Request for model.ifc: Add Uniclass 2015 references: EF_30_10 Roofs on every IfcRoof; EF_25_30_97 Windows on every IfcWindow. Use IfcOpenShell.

First a look at what the model holds.

```python
import ifcopenshell

model = ifcopenshell.open("model.ifc")
print(model.schema)
print("classifications:", [c.Name for c in model.by_type("IfcClassification")])
for ifc_class in ("IfcDoor", "IfcRoof", "IfcStair", "IfcWall", "IfcWindow"):
    print(ifc_class, len(model.by_type(ifc_class)))
```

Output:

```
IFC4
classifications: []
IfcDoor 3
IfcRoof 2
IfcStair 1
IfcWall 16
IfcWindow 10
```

```python
import ifcopenshell
import ifcopenshell.api.classification

model = ifcopenshell.open("model.ifc")

system = ifcopenshell.api.classification.add_classification(model, classification="Uniclass 2015")

codes = {
    "IfcRoof": ("EF_30_10", "Roofs"),
    "IfcWindow": ("EF_25_30_97", "Windows"),
}
for ifc_class, (code, name) in codes.items():
    products = model.by_type(ifc_class)
    ifcopenshell.api.classification.add_reference(
        model, products=products, classification=system, identification=code, name=name
    )
    print(code, len(products))

model.write("model_updated.ifc")
```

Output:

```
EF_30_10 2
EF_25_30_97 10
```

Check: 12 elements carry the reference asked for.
